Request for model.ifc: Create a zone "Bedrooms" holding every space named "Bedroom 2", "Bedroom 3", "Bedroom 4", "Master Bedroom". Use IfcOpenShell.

First a look at what the model holds.

```python
import ifcopenshell

model = ifcopenshell.open("model.ifc")
print(model.schema)
seen = {}
for space in model.by_type("IfcSpace"):
    seen[space.LongName] = seen.get(space.LongName, 0) + 1
for name, count in sorted(seen.items(), key=str):
    print(count, "x", name)
print("zones:", [z.Name for z in model.by_type("IfcZone")][:20])
```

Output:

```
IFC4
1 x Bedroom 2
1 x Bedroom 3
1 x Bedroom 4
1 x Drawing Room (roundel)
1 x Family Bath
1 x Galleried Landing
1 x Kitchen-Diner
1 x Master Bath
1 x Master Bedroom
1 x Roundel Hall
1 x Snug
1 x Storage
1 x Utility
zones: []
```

```python
import ifcopenshell
import ifcopenshell.api.group
import ifcopenshell.api.root

model = ifcopenshell.open("model.ifc")

names = {"Bedroom 2", "Bedroom 3", "Bedroom 4", "Master Bedroom"}
spaces = [s for s in model.by_type("IfcSpace") if s.LongName in names]

zone = ifcopenshell.api.root.create_entity(model, ifc_class="IfcZone", name="Bedrooms")
ifcopenshell.api.group.assign_group(model, products=spaces, group=zone)
print(len(spaces), "spaces in", zone.Name)

model.write("model_updated.ifc")
```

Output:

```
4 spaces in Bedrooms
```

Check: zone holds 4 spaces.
